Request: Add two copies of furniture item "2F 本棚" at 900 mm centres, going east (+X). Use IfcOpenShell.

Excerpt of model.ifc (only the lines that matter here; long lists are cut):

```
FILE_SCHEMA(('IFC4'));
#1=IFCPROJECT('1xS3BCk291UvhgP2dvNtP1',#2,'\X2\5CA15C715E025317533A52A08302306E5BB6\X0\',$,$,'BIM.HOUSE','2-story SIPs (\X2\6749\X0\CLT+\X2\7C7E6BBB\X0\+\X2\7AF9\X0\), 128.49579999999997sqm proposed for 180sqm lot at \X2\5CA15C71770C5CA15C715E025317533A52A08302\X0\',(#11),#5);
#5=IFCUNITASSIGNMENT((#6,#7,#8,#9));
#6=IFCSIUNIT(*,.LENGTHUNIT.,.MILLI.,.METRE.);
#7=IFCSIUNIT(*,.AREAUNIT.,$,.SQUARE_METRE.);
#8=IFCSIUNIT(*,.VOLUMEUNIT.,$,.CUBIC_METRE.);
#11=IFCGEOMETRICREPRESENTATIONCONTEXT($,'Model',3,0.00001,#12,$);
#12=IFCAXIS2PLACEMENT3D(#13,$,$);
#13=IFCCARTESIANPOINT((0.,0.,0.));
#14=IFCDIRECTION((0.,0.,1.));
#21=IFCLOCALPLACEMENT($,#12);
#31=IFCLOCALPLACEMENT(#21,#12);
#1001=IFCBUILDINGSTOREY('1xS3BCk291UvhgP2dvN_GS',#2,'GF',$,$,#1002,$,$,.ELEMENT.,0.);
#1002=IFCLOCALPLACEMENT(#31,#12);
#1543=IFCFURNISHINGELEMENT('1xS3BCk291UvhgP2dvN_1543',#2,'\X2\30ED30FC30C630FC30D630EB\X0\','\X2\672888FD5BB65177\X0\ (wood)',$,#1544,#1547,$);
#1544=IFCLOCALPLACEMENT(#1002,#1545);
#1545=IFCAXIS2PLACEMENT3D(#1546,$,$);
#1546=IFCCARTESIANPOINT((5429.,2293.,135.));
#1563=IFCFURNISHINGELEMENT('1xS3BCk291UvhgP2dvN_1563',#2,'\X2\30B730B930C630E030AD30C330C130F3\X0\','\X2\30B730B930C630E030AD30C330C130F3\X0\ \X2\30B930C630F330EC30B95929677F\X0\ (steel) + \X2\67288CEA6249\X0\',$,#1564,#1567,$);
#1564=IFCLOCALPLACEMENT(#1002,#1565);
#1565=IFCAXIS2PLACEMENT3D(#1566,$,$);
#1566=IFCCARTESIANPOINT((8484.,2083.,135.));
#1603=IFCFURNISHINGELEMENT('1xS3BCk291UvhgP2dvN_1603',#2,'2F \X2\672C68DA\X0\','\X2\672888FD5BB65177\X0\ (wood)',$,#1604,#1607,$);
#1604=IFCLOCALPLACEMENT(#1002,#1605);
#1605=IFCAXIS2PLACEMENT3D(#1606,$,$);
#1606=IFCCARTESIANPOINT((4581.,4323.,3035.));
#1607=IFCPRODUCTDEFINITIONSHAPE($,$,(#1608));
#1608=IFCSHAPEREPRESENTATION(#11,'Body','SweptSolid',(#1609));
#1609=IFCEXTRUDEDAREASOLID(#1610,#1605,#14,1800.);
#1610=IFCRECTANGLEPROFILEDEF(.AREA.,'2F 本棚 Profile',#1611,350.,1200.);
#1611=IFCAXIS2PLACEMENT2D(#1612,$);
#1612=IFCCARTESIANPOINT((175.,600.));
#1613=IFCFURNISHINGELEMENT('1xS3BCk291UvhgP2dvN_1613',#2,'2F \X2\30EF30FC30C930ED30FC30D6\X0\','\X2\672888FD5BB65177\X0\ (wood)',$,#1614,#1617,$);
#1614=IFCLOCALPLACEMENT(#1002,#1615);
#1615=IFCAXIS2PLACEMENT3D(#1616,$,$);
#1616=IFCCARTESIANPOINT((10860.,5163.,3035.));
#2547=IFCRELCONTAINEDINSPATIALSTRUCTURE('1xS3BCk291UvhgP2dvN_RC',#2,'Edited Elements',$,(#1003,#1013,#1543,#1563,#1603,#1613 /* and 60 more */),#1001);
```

```python
import numpy as np
import ifcopenshell
import ifcopenshell.api.geometry
import ifcopenshell.api.root
import ifcopenshell.util.element
import ifcopenshell.util.placement
import ifcopenshell.util.unit

model = ifcopenshell.open("model.ifc")
unit_scale = ifcopenshell.util.unit.calculate_unit_scale(model)


def reuse_history(source, copy):
    """copy_class also copies each property set's owner history, people and application; keep the originals."""
    for rel in copy.IsDefinedBy:
        if rel.is_a("IfcRelDefinesByProperties") and (history := rel.RelatingPropertyDefinition.OwnerHistory):
            rel.RelatingPropertyDefinition.OwnerHistory = source.OwnerHistory
            ifcopenshell.util.element.remove_deep2(model, history)


source = model.by_guid("1xS3BCk291UvhgP2dvN_1603")
base = ifcopenshell.util.placement.get_local_placement(source.ObjectPlacement)
step = np.array([1.0, 0.0, 0.0]) * 0.9 / unit_scale

for i in range(1, 3):
    copy = ifcopenshell.api.root.copy_class(model, product=source)
    copy.Representation = ifcopenshell.util.element.copy_deep(
        model, source.Representation, exclude=["IfcGeometricRepresentationContext", "IfcRepresentationMap"]
    )
    reuse_history(source, copy)
    matrix = base.copy()
    matrix[:3, 3] += i * step
    print("added at", matrix[:3, 3].round(3) + 0.0)
    ifcopenshell.api.geometry.edit_object_placement(model, product=copy, matrix=matrix, is_si=False)

model.write("model_v2.ifc")
```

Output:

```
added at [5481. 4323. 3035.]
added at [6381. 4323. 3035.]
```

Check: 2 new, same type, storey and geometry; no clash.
